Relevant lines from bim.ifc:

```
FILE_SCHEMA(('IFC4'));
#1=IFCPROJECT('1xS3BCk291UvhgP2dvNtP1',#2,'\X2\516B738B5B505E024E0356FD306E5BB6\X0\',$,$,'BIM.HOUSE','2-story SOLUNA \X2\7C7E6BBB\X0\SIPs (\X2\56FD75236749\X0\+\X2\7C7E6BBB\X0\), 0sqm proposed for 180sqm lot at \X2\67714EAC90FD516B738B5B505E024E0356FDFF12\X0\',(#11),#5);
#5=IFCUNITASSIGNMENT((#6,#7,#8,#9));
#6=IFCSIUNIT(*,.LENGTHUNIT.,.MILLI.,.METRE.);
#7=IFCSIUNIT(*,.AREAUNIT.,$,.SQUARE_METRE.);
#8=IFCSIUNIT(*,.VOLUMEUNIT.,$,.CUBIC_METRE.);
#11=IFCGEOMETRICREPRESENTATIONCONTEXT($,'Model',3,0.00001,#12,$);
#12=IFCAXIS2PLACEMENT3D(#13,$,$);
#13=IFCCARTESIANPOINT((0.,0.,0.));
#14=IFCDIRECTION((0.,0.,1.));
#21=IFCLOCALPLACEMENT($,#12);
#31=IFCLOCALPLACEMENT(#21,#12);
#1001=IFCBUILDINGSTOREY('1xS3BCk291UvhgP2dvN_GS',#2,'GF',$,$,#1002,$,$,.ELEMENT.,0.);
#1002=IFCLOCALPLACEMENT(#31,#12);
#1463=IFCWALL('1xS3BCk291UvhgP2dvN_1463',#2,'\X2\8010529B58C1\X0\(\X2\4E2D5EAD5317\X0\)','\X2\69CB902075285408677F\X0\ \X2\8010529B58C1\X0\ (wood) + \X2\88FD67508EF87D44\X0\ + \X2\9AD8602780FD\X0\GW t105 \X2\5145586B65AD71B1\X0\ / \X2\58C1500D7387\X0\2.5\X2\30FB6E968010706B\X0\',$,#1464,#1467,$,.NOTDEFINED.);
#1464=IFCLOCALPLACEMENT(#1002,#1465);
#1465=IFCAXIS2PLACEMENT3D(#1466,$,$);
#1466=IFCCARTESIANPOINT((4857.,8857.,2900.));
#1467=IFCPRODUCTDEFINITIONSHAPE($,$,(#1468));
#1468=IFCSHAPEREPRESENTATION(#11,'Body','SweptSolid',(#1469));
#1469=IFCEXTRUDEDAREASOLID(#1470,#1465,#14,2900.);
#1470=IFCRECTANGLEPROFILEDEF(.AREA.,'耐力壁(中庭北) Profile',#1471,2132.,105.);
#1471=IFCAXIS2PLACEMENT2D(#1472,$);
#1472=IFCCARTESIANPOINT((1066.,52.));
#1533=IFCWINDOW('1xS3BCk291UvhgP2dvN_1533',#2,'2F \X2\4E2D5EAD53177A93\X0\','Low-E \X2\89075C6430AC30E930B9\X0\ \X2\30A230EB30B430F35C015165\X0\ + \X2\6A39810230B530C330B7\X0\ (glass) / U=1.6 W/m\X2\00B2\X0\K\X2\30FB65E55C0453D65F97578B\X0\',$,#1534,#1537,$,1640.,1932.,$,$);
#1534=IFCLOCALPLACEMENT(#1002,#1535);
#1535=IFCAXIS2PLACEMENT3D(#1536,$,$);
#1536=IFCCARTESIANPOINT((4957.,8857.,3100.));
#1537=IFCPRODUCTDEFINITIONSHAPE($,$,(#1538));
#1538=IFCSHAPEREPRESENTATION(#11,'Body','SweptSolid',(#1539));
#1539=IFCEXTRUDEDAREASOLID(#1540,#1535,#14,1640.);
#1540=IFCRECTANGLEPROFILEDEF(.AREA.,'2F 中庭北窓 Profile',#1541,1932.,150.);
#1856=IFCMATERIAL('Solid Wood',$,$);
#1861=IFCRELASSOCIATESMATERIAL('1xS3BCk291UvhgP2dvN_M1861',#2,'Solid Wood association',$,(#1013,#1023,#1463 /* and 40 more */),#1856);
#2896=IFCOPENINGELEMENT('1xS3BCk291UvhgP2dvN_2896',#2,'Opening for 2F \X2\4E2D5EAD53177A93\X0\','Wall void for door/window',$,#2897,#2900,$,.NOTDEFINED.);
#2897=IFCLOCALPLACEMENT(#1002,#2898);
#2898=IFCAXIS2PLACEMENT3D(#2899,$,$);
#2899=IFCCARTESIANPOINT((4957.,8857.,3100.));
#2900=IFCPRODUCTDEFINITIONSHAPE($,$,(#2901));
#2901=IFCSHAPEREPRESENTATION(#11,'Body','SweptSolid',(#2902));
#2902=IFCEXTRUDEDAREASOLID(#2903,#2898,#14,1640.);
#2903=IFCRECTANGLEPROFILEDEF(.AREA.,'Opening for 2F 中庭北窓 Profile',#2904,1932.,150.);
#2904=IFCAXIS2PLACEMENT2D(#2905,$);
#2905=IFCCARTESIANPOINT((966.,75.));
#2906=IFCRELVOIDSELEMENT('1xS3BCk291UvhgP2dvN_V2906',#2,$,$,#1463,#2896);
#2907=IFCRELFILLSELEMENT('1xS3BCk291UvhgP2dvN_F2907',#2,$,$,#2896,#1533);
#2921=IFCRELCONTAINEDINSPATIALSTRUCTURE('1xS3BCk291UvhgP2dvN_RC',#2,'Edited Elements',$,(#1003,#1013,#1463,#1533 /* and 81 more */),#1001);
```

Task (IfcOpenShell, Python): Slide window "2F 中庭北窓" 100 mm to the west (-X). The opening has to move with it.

```python
import ifcopenshell
import ifcopenshell.api.geometry
import ifcopenshell.util.placement
import ifcopenshell.util.unit

model = ifcopenshell.open("bim.ifc")
unit_scale = ifcopenshell.util.unit.calculate_unit_scale(model)

window = model.by_id(1533)
opening = window.FillsVoids[0].RelatingOpeningElement
wall = opening.VoidsElements[0].RelatingBuildingElement

wall_matrix = ifcopenshell.util.placement.get_local_placement(wall.ObjectPlacement)
shift = wall_matrix[:3, 0] * -0.1 / unit_scale
before = ifcopenshell.util.placement.get_local_placement(window.ObjectPlacement)[:3, 3].copy()

# The window is not placed relative to its opening, so move both.
for product in (opening, window):
    matrix = ifcopenshell.util.placement.get_local_placement(product.ObjectPlacement)
    matrix[:3, 3] += shift
    ifcopenshell.api.geometry.edit_object_placement(model, product=product, matrix=matrix, is_si=False)

after = ifcopenshell.util.placement.get_local_placement(window.ObjectPlacement)[:3, 3]
print("window moved by", (after - before).round(3) + 0.0)

model.write("bim_edited.ifc")
```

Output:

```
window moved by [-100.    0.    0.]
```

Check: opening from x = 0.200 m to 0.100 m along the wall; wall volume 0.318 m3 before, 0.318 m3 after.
